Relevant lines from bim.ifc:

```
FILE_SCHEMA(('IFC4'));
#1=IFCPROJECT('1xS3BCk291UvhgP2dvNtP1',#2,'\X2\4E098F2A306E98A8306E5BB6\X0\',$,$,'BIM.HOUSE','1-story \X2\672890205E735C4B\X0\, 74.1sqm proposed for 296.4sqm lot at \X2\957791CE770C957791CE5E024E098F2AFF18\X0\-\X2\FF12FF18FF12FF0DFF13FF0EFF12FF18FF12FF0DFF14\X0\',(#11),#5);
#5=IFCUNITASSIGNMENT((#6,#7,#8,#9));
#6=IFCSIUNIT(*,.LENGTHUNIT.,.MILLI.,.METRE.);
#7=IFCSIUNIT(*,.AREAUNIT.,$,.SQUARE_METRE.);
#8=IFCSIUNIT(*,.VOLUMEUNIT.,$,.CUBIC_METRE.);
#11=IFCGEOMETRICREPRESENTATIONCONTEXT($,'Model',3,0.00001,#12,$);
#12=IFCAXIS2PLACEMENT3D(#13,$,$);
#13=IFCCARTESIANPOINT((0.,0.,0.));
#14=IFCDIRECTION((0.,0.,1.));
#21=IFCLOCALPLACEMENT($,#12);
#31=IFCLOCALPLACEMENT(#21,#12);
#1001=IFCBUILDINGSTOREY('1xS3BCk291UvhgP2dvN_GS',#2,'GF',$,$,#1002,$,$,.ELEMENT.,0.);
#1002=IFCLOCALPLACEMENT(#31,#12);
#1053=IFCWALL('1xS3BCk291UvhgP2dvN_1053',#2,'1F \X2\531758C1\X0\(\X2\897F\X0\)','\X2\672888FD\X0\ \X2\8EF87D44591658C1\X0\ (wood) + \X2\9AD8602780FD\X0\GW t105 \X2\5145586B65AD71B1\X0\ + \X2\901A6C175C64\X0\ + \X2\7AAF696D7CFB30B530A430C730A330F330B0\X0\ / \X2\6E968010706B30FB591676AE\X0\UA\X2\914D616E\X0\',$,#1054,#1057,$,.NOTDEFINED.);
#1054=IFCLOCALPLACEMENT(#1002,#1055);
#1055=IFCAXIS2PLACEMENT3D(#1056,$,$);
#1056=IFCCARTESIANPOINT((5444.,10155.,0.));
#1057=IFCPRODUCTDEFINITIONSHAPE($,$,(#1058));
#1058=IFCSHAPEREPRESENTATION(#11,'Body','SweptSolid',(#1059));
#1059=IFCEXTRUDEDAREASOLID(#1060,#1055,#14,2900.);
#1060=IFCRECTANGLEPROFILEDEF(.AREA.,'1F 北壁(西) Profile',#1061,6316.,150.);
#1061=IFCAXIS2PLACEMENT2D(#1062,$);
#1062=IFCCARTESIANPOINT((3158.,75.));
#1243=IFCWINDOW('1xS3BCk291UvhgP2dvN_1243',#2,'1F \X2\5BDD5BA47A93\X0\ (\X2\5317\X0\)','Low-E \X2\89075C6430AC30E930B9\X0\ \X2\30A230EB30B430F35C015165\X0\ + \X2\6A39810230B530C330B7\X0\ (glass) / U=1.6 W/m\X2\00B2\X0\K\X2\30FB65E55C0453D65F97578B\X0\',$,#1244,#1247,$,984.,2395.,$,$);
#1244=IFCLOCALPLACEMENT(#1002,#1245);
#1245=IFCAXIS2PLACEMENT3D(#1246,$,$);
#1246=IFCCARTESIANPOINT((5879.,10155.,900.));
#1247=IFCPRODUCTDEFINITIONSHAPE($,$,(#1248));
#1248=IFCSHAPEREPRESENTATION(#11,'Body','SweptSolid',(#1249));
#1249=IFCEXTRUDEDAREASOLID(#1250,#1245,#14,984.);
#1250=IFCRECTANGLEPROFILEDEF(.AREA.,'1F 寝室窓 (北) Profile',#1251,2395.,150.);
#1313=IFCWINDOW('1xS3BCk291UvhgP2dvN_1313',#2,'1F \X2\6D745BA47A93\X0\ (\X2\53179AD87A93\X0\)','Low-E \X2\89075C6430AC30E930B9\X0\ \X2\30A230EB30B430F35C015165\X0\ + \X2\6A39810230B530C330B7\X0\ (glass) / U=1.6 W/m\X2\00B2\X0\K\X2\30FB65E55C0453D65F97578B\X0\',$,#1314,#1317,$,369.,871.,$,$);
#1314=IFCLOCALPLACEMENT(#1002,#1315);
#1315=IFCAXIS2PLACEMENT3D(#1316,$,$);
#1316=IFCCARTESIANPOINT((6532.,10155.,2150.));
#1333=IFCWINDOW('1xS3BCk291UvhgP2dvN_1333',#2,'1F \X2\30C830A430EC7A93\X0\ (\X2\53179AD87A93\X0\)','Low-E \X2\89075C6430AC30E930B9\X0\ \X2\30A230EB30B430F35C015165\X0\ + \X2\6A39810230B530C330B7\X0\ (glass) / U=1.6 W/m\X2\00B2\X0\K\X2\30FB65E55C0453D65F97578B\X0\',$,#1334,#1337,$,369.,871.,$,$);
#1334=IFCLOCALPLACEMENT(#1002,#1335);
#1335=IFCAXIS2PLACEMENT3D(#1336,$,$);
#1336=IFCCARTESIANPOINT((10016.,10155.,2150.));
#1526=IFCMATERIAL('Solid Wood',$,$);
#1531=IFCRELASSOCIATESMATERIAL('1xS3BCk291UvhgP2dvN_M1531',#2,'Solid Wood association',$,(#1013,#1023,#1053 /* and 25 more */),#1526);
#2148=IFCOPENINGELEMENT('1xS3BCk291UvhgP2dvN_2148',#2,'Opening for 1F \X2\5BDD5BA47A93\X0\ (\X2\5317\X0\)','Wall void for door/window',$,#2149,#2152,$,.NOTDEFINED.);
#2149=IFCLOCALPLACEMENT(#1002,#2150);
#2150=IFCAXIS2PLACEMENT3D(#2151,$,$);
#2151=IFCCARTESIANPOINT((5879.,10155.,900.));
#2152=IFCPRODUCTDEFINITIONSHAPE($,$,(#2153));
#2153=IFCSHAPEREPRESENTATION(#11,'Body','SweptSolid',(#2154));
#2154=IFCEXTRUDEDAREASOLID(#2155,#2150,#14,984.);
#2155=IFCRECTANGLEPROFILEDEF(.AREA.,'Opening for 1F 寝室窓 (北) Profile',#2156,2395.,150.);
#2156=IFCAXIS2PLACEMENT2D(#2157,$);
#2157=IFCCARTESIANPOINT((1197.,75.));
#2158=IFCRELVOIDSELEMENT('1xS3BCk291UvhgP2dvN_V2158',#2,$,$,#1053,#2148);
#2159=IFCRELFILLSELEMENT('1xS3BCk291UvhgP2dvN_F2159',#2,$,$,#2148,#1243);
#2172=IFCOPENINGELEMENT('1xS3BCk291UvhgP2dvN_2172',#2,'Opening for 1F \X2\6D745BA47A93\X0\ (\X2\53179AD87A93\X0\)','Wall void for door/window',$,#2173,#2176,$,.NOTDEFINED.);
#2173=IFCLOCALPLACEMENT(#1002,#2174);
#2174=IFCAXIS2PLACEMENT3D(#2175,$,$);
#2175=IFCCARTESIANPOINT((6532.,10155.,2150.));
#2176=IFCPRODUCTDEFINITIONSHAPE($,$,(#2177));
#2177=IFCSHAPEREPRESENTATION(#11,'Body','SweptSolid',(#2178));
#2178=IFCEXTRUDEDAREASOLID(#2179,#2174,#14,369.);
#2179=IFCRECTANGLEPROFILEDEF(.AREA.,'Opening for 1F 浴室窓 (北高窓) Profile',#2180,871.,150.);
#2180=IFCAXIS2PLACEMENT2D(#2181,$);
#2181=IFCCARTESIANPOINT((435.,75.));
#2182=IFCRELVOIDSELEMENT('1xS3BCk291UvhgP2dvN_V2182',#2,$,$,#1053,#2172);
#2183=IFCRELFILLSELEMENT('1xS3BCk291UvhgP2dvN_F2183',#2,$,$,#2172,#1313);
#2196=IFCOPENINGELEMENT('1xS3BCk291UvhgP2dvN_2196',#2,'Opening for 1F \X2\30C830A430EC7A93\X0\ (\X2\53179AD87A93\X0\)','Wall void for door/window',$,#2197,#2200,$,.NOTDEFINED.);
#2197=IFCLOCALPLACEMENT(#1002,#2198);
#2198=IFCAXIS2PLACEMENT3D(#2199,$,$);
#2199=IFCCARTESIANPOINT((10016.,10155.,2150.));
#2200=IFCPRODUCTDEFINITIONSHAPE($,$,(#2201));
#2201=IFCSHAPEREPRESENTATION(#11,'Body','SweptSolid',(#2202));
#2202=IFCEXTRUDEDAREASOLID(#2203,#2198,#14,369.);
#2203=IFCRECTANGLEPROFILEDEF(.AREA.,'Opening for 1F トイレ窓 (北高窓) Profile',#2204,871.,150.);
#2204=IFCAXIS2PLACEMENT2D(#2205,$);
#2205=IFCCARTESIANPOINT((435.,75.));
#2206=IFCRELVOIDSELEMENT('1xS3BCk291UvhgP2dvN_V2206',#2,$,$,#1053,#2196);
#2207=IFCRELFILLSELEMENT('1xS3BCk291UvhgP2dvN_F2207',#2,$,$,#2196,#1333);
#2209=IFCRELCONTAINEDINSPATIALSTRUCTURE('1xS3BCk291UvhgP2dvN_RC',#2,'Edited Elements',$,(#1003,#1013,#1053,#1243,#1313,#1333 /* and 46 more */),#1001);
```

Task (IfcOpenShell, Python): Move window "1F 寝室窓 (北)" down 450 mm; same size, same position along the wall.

```python
import numpy as np
import ifcopenshell
import ifcopenshell.api.geometry
import ifcopenshell.util.placement
import ifcopenshell.util.unit

model = ifcopenshell.open("bim.ifc")
unit_scale = ifcopenshell.util.unit.calculate_unit_scale(model)

window = model.by_guid("1xS3BCk291UvhgP2dvN_1243")
opening = window.FillsVoids[0].RelatingOpeningElement
dz = -0.45 / unit_scale

shift = np.array([0.0, 0.0, dz])
# The window is not placed relative to its opening, so move both.
for product in (opening, window):
    matrix = ifcopenshell.util.placement.get_local_placement(product.ObjectPlacement)
    matrix[:3, 3] += shift
    ifcopenshell.api.geometry.edit_object_placement(model, product=product, matrix=matrix, is_si=False)

print(f"moved by {dz * unit_scale:+.3f} m")

model.write("bim-out.ifc")
```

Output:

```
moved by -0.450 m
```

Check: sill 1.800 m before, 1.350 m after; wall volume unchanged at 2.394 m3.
